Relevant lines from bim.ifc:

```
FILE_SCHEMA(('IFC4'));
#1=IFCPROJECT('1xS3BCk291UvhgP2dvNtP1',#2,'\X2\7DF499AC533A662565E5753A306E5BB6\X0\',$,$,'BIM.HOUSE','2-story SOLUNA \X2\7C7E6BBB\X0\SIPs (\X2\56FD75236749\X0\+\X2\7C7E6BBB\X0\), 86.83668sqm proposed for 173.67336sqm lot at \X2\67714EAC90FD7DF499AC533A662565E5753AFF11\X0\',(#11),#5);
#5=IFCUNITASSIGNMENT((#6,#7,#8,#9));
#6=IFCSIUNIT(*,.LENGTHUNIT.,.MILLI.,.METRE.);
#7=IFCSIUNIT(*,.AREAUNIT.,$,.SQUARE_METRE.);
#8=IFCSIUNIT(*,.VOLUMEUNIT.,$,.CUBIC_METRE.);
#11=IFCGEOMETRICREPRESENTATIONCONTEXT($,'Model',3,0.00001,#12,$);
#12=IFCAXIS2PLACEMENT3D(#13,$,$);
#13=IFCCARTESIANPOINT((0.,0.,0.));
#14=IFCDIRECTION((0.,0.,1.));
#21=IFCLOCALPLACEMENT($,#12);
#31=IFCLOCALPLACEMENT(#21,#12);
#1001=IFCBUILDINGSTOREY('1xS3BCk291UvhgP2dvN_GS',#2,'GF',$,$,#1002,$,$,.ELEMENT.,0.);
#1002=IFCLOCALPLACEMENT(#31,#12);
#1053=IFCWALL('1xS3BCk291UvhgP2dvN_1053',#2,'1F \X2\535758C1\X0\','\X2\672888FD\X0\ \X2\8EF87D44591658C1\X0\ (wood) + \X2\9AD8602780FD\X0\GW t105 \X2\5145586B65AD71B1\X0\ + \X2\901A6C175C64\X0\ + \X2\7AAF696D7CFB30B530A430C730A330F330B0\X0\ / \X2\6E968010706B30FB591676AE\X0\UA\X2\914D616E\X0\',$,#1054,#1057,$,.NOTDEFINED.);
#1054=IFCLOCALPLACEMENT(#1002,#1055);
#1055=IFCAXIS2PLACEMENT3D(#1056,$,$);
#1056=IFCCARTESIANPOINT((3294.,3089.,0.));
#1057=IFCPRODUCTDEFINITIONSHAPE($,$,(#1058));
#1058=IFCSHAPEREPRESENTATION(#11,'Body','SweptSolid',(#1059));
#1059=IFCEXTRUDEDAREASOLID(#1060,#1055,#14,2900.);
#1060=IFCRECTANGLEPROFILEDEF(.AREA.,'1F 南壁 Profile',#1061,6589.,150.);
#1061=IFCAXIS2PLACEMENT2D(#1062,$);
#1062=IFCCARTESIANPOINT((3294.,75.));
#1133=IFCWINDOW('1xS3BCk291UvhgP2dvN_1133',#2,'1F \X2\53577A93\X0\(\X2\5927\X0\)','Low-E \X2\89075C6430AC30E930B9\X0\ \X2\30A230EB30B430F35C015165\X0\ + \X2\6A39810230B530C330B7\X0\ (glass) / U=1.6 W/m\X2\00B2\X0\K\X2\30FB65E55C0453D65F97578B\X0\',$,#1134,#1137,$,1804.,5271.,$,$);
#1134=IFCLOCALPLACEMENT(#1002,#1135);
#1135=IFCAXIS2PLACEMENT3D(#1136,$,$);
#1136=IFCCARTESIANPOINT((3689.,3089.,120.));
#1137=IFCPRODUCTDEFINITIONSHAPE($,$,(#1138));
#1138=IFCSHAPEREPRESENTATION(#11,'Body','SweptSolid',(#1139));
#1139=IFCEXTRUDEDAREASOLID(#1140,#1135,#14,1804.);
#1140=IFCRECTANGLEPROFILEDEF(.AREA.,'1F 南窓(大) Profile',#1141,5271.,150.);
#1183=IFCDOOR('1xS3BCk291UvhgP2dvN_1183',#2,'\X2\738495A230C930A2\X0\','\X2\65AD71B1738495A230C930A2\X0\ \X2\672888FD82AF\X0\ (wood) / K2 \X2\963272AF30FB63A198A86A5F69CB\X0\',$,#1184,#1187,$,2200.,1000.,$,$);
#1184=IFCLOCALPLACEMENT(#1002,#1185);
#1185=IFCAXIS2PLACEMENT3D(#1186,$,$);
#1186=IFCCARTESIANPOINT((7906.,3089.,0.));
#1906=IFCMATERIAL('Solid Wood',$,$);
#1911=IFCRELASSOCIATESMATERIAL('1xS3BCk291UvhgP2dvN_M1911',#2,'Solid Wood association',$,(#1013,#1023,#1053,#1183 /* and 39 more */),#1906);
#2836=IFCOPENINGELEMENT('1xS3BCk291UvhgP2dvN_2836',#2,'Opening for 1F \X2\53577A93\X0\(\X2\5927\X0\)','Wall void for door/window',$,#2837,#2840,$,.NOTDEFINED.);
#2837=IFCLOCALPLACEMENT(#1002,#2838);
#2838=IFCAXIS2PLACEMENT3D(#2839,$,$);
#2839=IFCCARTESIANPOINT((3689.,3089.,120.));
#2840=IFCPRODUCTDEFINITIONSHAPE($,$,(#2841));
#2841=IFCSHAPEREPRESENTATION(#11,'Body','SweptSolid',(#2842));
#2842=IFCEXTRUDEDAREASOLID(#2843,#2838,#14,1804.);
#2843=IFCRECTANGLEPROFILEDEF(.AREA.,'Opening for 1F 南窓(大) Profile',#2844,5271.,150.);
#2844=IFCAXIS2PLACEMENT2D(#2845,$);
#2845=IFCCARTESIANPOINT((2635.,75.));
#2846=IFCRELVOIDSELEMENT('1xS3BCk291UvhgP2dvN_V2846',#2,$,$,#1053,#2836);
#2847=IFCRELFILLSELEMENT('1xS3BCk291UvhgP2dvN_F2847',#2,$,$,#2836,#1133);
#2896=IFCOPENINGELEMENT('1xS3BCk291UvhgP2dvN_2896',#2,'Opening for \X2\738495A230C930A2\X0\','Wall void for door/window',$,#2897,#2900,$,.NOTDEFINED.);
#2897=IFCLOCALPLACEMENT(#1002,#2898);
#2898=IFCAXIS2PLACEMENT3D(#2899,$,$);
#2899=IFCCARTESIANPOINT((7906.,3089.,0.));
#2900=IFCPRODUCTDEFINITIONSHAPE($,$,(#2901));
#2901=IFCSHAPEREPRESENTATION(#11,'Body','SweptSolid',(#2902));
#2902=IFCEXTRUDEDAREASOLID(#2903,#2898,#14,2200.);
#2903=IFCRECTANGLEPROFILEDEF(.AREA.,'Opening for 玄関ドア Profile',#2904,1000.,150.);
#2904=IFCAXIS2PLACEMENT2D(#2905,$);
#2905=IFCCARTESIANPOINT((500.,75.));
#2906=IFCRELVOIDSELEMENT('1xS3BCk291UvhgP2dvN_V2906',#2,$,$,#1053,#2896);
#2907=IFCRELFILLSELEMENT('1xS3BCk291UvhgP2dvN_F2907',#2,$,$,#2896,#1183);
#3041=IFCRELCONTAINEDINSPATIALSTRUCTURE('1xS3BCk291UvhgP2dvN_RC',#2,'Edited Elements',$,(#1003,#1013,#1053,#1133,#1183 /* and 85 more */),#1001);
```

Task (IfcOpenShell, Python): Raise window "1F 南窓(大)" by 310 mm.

```python
import numpy as np
import ifcopenshell
import ifcopenshell.api.geometry
import ifcopenshell.util.placement
import ifcopenshell.util.unit

model = ifcopenshell.open("bim.ifc")
unit_scale = ifcopenshell.util.unit.calculate_unit_scale(model)

window = model.by_guid("1xS3BCk291UvhgP2dvN_1133")
opening = window.FillsVoids[0].RelatingOpeningElement
dz = 310.0

shift = np.array([0.0, 0.0, dz])
# The window is not placed relative to its opening, so move both.
for product in (opening, window):
    matrix = ifcopenshell.util.placement.get_local_placement(product.ObjectPlacement)
    matrix[:3, 3] += shift
    ifcopenshell.api.geometry.edit_object_placement(model, product=product, matrix=matrix, is_si=False)

print(f"moved by {dz * unit_scale:+.3f} m")

model.write("bim-out.ifc")
```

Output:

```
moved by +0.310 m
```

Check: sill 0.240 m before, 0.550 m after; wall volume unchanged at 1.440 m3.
